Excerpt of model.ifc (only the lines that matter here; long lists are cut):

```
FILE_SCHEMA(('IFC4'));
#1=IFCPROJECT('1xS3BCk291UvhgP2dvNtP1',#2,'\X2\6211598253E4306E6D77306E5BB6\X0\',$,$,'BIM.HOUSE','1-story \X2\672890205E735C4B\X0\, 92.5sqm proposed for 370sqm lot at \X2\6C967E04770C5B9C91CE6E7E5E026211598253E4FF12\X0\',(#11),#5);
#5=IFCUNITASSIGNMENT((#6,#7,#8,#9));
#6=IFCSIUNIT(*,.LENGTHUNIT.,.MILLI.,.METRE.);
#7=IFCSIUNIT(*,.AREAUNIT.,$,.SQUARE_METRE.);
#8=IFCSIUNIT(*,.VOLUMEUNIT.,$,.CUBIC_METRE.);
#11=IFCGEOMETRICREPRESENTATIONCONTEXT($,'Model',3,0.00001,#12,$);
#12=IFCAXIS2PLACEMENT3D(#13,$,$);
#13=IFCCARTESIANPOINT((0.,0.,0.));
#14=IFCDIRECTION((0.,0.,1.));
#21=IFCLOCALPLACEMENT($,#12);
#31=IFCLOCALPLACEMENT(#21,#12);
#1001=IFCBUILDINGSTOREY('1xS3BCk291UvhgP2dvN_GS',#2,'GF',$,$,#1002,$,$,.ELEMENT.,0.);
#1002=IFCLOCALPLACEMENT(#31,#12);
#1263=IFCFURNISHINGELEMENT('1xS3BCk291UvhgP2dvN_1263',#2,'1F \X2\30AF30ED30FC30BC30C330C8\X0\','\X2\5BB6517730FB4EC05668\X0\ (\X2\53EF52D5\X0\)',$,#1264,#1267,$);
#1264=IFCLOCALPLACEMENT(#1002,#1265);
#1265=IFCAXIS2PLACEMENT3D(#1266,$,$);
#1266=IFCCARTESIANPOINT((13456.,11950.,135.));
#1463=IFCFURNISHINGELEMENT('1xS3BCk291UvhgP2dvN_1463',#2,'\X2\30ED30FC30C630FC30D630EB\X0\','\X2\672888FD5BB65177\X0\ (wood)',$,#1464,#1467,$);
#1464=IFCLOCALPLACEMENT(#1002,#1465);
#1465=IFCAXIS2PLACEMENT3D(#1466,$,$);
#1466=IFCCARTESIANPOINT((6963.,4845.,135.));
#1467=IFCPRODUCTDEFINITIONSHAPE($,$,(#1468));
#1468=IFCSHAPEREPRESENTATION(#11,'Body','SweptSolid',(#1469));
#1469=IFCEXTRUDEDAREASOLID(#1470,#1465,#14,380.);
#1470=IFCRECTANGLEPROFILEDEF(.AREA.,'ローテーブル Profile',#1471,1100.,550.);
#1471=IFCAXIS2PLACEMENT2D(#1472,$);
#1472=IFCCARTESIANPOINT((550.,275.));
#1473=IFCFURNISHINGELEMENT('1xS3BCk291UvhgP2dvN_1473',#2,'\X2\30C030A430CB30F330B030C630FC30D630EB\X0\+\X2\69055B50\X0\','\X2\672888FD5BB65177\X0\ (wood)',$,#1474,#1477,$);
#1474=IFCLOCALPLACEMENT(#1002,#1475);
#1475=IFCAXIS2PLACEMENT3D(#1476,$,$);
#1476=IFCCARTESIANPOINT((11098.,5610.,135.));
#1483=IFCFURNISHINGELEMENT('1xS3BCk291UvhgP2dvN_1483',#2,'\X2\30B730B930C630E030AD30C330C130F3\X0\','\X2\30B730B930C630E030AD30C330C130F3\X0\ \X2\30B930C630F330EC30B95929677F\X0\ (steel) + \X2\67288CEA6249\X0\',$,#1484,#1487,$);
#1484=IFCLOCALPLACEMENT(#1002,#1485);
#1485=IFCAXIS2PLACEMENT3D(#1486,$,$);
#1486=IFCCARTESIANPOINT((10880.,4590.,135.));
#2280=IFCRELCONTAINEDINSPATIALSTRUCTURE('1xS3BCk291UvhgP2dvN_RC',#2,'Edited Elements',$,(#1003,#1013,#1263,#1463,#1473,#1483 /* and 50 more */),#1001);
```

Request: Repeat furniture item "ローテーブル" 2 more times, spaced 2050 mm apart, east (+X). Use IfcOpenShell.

```python
import numpy as np
import ifcopenshell
import ifcopenshell.api.geometry
import ifcopenshell.api.root
import ifcopenshell.util.element
import ifcopenshell.util.placement
import ifcopenshell.util.unit

model = ifcopenshell.open("model.ifc")
unit_scale = ifcopenshell.util.unit.calculate_unit_scale(model)


def reuse_history(source, copy):
    """copy_class also copies each property set's owner history, people and application; keep the originals."""
    for rel in copy.IsDefinedBy:
        if rel.is_a("IfcRelDefinesByProperties") and (history := rel.RelatingPropertyDefinition.OwnerHistory):
            rel.RelatingPropertyDefinition.OwnerHistory = source.OwnerHistory
            ifcopenshell.util.element.remove_deep2(model, history)


source = model.by_id(1463)
base = ifcopenshell.util.placement.get_local_placement(source.ObjectPlacement)
step = np.array([1.0, 0.0, 0.0]) * 2.05 / unit_scale

for i in range(1, 3):
    copy = ifcopenshell.api.root.copy_class(model, product=source)
    copy.Representation = ifcopenshell.util.element.copy_deep(
        model, source.Representation, exclude=["IfcGeometricRepresentationContext", "IfcRepresentationMap"]
    )
    reuse_history(source, copy)
    matrix = base.copy()
    matrix[:3, 3] += i * step
    print("added at", matrix[:3, 3].round(3) + 0.0)
    ifcopenshell.api.geometry.edit_object_placement(model, product=copy, matrix=matrix, is_si=False)

model.write("model-out.ifc")
```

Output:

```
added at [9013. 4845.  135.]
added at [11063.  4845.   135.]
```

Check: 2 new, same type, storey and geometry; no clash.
